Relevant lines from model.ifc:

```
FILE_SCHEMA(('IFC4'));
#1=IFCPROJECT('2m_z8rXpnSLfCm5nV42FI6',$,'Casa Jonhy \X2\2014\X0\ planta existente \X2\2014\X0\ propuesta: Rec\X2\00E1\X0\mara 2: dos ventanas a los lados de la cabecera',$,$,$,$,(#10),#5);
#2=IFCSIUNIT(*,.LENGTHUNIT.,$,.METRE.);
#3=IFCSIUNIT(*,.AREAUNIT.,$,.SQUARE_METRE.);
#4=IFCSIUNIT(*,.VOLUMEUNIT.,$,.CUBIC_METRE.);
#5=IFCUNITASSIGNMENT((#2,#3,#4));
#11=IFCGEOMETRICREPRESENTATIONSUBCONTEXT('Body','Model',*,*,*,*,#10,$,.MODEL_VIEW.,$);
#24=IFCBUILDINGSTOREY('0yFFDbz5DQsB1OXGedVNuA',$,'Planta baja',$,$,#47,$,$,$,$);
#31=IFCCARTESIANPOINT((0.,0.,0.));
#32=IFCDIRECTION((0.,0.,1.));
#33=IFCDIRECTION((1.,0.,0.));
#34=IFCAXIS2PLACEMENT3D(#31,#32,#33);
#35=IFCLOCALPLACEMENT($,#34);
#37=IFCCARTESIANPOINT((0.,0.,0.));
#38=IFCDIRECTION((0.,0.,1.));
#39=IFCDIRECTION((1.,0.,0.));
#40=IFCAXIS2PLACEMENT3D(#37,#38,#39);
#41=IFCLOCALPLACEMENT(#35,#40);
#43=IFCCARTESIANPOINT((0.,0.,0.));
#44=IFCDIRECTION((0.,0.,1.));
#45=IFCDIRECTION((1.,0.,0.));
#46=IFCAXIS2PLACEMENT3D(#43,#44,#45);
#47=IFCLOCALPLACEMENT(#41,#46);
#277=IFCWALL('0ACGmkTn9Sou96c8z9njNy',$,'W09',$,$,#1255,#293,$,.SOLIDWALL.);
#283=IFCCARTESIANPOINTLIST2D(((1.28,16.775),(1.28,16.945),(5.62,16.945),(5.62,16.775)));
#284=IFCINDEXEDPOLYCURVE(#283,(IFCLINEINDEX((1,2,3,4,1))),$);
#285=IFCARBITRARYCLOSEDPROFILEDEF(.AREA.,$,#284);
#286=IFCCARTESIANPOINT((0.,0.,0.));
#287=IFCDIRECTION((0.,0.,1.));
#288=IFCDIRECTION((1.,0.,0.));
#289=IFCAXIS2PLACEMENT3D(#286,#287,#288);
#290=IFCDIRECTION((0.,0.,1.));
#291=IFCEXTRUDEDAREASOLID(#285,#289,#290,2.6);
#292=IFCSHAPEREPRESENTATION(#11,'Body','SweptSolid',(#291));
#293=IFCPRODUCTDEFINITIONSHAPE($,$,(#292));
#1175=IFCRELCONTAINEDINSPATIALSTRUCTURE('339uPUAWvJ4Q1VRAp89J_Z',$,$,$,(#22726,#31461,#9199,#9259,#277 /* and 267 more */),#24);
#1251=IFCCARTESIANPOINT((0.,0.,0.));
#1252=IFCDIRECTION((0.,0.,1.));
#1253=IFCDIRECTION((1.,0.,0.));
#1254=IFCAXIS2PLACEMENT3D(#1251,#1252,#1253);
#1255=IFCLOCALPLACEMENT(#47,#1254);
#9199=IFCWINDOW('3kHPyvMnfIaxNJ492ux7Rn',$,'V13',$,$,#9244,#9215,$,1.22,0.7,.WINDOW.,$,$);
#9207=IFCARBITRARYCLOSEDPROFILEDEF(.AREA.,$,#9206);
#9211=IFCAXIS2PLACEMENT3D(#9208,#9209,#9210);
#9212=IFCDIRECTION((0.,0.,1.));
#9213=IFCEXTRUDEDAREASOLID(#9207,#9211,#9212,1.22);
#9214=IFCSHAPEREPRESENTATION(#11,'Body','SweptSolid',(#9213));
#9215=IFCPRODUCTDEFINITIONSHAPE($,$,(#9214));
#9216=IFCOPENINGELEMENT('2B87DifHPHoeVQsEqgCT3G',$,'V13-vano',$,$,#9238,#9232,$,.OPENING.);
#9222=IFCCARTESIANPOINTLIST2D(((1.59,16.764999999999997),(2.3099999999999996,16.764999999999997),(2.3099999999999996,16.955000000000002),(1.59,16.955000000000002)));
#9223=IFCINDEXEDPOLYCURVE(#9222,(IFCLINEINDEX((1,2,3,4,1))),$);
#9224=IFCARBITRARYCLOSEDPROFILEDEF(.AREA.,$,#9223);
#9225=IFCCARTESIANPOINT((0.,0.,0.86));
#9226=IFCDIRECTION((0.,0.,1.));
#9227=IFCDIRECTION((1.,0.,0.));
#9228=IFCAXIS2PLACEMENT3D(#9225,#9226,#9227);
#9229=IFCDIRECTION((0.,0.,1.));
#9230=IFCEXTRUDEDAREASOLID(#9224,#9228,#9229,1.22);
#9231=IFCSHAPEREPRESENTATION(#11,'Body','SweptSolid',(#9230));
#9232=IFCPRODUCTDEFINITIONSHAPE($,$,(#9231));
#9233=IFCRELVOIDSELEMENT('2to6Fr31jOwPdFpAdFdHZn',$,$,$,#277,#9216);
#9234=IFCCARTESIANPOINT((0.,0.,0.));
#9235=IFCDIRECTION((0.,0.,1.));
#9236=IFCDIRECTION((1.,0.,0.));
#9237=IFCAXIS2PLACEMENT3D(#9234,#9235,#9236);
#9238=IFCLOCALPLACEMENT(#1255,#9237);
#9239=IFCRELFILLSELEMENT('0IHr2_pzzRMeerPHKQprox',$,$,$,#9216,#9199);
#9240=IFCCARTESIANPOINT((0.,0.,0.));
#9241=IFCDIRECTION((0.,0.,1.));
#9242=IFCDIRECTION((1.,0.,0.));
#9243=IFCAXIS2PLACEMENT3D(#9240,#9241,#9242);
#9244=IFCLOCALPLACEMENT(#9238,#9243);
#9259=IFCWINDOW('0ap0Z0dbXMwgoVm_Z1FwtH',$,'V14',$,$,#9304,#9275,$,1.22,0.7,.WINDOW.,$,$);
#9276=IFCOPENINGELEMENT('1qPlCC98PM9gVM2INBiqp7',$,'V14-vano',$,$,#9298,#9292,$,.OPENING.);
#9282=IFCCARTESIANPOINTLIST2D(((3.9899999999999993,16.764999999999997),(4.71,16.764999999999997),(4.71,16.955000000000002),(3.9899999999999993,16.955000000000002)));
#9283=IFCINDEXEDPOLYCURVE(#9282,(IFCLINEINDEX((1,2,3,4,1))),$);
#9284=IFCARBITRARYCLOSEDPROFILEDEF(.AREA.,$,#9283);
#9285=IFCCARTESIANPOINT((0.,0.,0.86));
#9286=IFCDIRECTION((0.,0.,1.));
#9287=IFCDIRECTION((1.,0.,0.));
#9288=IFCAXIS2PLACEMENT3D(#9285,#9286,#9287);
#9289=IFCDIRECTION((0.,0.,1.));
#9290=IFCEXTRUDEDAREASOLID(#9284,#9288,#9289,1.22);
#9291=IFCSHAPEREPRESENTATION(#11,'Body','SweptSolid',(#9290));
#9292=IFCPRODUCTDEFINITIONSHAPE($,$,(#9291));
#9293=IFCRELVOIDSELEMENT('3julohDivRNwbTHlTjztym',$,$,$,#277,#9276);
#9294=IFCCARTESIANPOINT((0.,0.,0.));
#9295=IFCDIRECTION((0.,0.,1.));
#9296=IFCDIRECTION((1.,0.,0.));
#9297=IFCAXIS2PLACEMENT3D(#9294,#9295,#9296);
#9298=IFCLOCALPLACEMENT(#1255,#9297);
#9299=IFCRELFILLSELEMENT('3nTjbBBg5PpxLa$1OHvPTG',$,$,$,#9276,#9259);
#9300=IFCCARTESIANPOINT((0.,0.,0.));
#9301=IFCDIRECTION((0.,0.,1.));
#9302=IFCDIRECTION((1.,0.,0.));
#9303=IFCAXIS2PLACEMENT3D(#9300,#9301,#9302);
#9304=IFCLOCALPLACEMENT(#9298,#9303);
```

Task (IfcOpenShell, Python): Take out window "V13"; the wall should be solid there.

```python
import ifcopenshell
import ifcopenshell.api.feature
import ifcopenshell.api.root
import ifcopenshell.geom
import ifcopenshell.util.shape

model = ifcopenshell.open("model.ifc")
settings = ifcopenshell.geom.settings()


def volume(element):
    """Net volume in cubic metres, openings subtracted."""
    shape = ifcopenshell.geom.create_shape(settings, element)
    return ifcopenshell.util.shape.get_volume(shape.geometry)


window = model.by_guid("3kHPyvMnfIaxNJ492ux7Rn")
opening = window.FillsVoids[0].RelatingOpeningElement
wall = opening.VoidsElements[0].RelatingBuildingElement
before = volume(wall)

ifcopenshell.api.root.remove_product(model, product=window)
ifcopenshell.api.feature.remove_feature(model, feature=opening)

after = volume(wall)

print(f"wall volume {before:.3f} -> {after:.3f} m3")

model.write("model-out.ifc")
```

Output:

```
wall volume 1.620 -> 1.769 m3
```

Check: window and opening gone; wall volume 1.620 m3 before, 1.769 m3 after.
